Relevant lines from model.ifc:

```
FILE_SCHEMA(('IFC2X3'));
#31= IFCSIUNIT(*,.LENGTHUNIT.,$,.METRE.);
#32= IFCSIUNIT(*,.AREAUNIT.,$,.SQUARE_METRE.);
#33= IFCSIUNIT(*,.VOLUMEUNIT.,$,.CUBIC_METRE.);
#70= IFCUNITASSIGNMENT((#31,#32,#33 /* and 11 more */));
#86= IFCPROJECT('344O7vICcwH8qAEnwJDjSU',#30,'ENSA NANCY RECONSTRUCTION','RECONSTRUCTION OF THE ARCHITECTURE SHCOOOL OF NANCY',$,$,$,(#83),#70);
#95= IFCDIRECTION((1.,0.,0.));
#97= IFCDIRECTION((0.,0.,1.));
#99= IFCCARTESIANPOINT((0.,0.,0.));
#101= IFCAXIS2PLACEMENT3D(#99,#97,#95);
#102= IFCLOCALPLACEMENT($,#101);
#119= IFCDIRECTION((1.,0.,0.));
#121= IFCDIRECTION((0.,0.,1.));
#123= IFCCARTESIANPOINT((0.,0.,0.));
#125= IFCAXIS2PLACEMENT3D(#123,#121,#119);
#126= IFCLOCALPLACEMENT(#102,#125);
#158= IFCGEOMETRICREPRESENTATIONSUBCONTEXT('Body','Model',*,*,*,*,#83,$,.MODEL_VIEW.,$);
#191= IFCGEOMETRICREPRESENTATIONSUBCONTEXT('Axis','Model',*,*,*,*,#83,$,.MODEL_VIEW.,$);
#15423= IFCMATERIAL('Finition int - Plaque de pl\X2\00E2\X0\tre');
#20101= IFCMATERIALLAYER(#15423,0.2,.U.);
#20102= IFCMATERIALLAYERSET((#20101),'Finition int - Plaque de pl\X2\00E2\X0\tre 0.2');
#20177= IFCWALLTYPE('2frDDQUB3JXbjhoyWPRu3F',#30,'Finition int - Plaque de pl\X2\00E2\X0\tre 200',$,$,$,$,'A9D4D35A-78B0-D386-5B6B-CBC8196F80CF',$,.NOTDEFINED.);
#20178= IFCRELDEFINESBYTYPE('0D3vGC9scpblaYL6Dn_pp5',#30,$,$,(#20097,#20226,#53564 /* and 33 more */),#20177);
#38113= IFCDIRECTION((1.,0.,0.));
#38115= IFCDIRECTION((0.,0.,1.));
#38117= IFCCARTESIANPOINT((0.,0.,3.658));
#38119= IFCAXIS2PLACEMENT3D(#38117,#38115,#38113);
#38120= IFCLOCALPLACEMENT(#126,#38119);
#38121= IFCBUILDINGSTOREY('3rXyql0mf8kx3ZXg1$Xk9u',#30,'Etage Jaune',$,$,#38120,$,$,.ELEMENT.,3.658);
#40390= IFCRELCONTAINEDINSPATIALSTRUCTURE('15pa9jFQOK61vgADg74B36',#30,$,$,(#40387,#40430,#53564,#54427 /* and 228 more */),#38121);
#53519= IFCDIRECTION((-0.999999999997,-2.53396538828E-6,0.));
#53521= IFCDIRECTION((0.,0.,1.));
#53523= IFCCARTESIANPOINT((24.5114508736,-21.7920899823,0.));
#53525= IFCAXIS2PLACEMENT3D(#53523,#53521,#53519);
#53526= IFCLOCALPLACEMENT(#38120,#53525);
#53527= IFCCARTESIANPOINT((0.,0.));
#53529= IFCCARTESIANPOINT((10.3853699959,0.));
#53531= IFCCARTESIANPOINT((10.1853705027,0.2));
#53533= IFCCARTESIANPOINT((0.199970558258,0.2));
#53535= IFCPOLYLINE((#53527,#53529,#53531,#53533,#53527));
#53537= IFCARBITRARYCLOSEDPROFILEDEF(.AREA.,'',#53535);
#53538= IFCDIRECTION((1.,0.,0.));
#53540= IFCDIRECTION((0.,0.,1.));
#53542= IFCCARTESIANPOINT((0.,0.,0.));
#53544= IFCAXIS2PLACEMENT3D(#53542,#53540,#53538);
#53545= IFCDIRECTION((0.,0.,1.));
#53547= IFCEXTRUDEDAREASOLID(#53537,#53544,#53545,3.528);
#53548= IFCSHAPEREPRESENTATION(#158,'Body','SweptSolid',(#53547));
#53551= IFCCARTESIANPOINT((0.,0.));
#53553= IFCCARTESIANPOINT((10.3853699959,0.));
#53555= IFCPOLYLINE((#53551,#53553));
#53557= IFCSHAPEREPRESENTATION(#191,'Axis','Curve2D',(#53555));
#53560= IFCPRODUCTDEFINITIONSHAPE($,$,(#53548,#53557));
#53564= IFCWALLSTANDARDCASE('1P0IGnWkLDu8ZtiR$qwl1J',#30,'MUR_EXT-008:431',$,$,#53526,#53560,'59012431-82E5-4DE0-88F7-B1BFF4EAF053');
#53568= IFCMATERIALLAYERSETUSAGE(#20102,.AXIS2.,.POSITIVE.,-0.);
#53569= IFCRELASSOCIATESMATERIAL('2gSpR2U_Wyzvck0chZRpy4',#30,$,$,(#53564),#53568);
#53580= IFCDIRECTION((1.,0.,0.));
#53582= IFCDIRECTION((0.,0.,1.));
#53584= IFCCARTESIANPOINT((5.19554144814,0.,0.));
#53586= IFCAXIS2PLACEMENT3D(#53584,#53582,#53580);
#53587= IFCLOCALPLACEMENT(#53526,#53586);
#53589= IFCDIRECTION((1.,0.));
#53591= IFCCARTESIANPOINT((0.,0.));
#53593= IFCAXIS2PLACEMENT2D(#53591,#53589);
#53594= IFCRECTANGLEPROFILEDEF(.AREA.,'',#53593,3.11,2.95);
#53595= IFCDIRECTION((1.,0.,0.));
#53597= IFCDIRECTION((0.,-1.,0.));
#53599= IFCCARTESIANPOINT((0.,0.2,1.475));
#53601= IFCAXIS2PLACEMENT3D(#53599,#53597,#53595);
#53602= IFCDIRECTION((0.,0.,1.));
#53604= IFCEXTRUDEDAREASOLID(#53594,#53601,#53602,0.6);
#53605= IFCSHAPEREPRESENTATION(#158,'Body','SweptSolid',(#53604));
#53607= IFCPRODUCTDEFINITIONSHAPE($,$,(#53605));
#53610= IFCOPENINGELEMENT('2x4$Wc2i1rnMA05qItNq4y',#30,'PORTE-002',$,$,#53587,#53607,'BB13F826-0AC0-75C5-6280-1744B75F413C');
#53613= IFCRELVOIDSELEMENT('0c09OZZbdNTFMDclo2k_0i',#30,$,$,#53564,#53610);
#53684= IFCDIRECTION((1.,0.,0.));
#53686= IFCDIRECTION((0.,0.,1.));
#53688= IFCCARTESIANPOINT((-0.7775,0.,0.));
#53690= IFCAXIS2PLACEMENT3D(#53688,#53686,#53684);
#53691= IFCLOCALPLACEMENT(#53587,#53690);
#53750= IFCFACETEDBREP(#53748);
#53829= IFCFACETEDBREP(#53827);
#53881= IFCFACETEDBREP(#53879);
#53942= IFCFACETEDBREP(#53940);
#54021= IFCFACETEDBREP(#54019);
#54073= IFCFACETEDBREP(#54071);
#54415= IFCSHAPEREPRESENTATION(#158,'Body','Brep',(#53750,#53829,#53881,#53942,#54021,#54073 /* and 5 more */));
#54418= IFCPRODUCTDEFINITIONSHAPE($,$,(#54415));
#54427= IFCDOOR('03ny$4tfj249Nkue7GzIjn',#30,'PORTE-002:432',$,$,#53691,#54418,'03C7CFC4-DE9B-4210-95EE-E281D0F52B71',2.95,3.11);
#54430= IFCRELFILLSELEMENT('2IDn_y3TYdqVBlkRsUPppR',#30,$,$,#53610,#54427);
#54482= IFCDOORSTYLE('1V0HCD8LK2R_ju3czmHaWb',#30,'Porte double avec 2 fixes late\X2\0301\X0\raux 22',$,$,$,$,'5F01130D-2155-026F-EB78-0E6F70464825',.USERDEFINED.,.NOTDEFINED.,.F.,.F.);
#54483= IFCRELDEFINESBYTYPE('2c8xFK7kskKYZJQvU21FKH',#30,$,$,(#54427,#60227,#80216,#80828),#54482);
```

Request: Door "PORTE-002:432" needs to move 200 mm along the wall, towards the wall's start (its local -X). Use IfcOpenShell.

```python
import ifcopenshell
import ifcopenshell.api.geometry
import ifcopenshell.util.placement
import ifcopenshell.util.unit

model = ifcopenshell.open("model.ifc")
unit_scale = ifcopenshell.util.unit.calculate_unit_scale(model)

door = model.by_guid("03ny$4tfj249Nkue7GzIjn")
opening = door.FillsVoids[0].RelatingOpeningElement
wall = opening.VoidsElements[0].RelatingBuildingElement

wall_matrix = ifcopenshell.util.placement.get_local_placement(wall.ObjectPlacement)
shift = wall_matrix[:3, 0] * -0.2 / unit_scale
before = ifcopenshell.util.placement.get_local_placement(door.ObjectPlacement)[:3, 3].copy()

# The door is placed relative to its opening, so it follows when the opening moves.
matrix = ifcopenshell.util.placement.get_local_placement(opening.ObjectPlacement)
matrix[:3, 3] += shift
ifcopenshell.api.geometry.edit_object_placement(
    model, product=opening, matrix=matrix, is_si=False, should_transform_children=True
)

after = ifcopenshell.util.placement.get_local_placement(door.ObjectPlacement)[:3, 3]
print("door moved by", (after - before).round(3) + 0.0)

model.write("model_updated.ifc")
```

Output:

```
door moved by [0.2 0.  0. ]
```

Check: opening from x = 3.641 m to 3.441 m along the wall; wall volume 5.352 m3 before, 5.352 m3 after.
